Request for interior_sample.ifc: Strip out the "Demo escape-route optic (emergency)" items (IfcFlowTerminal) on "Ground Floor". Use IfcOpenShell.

First a look at what the model holds.

```python
import ifcopenshell
import ifcopenshell.util.element

model = ifcopenshell.open("interior_sample.ifc")
print(model.schema)
storey = next(s for s in model.by_type("IfcBuildingStorey") if s.Name == "Ground Floor")
terminals = [e for e in ifcopenshell.util.element.get_decomposition(storey) if e.is_a("IfcFlowTerminal")]
seen = {}
for e in terminals:
    element_type = ifcopenshell.util.element.get_type(e)
    name = element_type.Name if element_type not in (None, e) else None
    seen[name] = seen.get(name, 0) + 1
for name, count in sorted(seen.items(), key=str):
    print(count, "x", name)
```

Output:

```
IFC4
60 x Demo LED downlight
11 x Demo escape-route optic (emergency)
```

```python
import ifcopenshell
import ifcopenshell.api.root
import ifcopenshell.util.element

model = ifcopenshell.open("interior_sample.ifc")

storey = next(s for s in model.by_type("IfcBuildingStorey") if s.Name == "Ground Floor")
terminals = [e for e in ifcopenshell.util.element.get_decomposition(storey) if e.is_a("IfcFlowTerminal")]
targets = [e for e in terminals if (t := ifcopenshell.util.element.get_type(e)) not in (None, e) and t.Name == "Demo escape-route optic (emergency)"]

for e in targets:
    ifcopenshell.api.root.remove_product(model, product=e)
print(len(targets), "removed")

model.write("interior_sample-out.ifc")
```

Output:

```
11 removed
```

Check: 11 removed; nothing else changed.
